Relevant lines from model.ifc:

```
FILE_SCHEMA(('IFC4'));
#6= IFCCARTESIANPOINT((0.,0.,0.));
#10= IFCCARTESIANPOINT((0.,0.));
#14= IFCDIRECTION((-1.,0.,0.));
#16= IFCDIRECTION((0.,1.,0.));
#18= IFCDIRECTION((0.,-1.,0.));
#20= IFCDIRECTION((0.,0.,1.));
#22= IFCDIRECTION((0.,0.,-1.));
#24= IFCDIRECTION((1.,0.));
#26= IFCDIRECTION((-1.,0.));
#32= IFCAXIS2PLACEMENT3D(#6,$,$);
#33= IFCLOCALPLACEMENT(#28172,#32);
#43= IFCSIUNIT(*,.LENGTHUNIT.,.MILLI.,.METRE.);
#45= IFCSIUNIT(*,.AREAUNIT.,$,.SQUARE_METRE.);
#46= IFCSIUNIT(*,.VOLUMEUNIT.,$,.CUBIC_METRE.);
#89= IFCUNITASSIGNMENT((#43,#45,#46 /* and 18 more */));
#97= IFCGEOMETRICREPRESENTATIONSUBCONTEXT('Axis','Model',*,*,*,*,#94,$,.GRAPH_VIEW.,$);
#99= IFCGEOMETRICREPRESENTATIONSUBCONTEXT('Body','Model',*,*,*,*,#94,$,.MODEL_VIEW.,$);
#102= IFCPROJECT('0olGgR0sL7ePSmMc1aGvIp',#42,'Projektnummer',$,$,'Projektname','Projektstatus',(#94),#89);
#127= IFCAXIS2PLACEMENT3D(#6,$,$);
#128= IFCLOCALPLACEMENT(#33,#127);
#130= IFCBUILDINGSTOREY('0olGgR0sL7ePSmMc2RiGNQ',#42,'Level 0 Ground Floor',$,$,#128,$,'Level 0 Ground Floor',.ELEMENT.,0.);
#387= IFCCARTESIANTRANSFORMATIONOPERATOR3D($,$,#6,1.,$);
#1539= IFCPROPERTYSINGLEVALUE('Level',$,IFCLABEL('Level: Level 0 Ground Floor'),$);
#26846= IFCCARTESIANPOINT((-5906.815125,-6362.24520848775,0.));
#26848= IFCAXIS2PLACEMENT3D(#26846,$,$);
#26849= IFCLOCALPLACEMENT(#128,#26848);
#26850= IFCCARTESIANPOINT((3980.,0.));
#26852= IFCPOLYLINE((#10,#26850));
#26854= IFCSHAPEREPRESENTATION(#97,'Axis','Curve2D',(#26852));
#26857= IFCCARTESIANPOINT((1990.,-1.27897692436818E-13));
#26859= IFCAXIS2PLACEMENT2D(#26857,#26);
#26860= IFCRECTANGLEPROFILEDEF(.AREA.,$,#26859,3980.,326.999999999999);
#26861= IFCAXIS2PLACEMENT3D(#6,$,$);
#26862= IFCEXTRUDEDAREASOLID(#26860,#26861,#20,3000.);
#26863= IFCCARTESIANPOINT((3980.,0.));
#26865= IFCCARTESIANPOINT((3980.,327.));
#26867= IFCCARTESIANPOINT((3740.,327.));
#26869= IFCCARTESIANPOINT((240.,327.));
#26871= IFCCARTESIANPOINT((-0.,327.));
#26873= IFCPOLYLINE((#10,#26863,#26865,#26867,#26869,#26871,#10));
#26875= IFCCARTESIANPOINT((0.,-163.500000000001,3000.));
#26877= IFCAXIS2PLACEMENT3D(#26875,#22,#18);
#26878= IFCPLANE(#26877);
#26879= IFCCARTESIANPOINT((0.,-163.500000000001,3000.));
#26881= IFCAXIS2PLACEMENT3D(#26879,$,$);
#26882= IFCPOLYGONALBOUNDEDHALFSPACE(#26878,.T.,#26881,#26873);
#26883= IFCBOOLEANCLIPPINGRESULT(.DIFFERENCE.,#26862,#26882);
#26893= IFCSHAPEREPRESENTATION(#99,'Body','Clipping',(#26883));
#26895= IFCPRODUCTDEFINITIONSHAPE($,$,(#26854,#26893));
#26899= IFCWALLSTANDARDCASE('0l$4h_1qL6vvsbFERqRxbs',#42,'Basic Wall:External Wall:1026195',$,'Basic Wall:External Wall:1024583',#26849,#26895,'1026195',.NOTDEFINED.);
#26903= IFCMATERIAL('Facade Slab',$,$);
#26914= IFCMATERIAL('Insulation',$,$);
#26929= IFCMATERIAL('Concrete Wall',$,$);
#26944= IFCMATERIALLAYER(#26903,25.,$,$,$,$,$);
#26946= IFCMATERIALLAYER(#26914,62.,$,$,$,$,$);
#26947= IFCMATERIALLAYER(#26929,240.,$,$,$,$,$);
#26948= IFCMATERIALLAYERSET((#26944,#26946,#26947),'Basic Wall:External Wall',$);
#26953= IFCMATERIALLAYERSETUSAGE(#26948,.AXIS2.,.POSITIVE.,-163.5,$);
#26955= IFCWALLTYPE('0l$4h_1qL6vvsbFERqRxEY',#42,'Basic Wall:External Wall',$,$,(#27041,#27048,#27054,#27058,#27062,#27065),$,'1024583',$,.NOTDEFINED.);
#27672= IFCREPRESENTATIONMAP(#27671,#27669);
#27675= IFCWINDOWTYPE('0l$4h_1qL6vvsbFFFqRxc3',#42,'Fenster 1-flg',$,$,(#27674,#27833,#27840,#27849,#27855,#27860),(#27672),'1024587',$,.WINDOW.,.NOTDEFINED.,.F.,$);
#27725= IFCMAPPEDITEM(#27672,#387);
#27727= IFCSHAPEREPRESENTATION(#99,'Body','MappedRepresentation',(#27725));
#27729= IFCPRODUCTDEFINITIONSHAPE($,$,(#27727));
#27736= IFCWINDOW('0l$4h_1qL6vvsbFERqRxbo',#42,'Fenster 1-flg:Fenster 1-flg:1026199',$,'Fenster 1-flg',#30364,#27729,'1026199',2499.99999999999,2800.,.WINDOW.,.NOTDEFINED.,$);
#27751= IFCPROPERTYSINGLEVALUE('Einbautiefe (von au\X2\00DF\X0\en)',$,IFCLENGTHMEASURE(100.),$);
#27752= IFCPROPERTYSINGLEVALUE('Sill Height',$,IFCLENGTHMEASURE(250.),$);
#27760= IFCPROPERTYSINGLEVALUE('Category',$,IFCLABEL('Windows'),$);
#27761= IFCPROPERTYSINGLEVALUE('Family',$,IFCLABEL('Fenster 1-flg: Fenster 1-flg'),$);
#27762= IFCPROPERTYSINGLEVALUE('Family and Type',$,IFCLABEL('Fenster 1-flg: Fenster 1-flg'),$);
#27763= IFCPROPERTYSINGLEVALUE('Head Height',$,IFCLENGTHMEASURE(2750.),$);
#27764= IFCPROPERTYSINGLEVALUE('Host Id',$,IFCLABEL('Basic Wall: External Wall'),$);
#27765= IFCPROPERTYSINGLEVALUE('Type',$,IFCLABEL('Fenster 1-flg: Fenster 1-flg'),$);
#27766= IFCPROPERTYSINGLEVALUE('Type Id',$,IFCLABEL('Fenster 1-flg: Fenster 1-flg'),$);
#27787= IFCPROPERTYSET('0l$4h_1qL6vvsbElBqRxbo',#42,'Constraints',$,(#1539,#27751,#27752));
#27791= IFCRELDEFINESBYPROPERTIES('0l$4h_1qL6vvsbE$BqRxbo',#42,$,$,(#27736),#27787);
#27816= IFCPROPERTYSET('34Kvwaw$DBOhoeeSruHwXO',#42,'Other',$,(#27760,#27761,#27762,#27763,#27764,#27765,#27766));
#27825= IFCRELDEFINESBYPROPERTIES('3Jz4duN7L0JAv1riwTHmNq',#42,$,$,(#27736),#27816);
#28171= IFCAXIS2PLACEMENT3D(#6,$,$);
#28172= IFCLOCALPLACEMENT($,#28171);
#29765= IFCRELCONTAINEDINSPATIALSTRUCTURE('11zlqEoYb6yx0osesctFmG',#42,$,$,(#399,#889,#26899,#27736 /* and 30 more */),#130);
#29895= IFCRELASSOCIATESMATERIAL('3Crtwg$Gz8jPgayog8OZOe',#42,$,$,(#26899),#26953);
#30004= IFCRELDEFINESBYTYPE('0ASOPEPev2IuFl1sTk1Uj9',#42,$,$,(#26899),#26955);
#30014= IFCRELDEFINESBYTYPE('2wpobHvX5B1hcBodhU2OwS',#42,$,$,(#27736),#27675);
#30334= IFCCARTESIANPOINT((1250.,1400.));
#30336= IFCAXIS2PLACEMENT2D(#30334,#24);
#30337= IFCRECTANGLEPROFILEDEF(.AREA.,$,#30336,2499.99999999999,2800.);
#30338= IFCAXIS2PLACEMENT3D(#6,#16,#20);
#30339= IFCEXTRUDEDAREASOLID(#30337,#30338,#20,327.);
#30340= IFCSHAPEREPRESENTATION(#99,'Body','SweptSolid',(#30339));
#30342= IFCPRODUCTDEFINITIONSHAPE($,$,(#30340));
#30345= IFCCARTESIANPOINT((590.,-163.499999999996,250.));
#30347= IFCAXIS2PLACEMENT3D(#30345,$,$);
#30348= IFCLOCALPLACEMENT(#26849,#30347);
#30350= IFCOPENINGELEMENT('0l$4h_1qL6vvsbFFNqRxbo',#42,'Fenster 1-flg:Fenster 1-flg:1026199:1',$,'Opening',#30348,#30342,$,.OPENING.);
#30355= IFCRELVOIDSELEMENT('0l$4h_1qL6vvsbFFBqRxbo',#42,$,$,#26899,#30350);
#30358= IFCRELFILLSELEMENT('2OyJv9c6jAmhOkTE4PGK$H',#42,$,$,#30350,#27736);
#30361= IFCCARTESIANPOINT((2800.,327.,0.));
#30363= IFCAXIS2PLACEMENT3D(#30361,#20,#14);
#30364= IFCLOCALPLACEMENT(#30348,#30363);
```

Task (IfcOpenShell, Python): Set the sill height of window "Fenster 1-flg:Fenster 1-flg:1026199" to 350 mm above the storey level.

```python
import numpy as np
import ifcopenshell
import ifcopenshell.api.geometry
import ifcopenshell.api.pset
import ifcopenshell.geom
import ifcopenshell.util.element
import ifcopenshell.util.placement
import ifcopenshell.util.shape
import ifcopenshell.util.unit

model = ifcopenshell.open("model.ifc")
unit_scale = ifcopenshell.util.unit.calculate_unit_scale(model)

window = model.by_guid("0l$4h_1qL6vvsbFERqRxbo")
opening = window.FillsVoids[0].RelatingOpeningElement
storey = ifcopenshell.util.element.get_container(window, ifc_class="IfcBuildingStorey")
level = ifcopenshell.util.placement.get_local_placement(storey.ObjectPlacement)[2, 3]

# The opening's origin need not be at the sill, so measure its lowest point.
shape = ifcopenshell.geom.create_shape(ifcopenshell.geom.settings(), opening)
bottom = ifcopenshell.util.shape.get_shape_bottom_elevation(shape, shape.geometry) / unit_scale
dz = level + 0.35 / unit_scale - bottom

shift = np.array([0.0, 0.0, dz])
# The window is placed relative to its opening, so it follows when the opening moves.
matrix = ifcopenshell.util.placement.get_local_placement(opening.ObjectPlacement)
matrix[:3, 3] += shift
ifcopenshell.api.geometry.edit_object_placement(
    model, product=opening, matrix=matrix, is_si=False, should_transform_children=True
)

# Keep the stored heights in step.
pset = model.by_id(ifcopenshell.util.element.get_pset(window, "Constraints", should_inherit=False)["id"])
ifcopenshell.api.pset.edit_pset(model, pset=pset, properties={
    "Sill Height": model.create_entity("IfcLengthMeasure", ifcopenshell.util.element.get_pset(window, "Constraints", "Sill Height") + dz),
})
pset = model.by_id(ifcopenshell.util.element.get_pset(window, "Other", should_inherit=False)["id"])
ifcopenshell.api.pset.edit_pset(model, pset=pset, properties={
    "Head Height": model.create_entity("IfcLengthMeasure", ifcopenshell.util.element.get_pset(window, "Other", "Head Height") + dz),
})

print(f"moved by {dz * unit_scale:+.3f} m")

model.write("model_v2.ifc")
```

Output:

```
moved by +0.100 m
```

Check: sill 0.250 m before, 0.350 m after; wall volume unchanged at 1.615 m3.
